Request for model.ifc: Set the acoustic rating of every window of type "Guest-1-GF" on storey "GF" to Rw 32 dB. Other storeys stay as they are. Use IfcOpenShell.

First a look at what the model holds.

```python
import ifcopenshell
import ifcopenshell.util.element

model = ifcopenshell.open("model.ifc")
print(model.schema)
storey = next(s for s in model.by_type("IfcBuildingStorey") if s.Name == "GF")
windows = [e for e in ifcopenshell.util.element.get_decomposition(storey) if e.is_a("IfcWindow")]
seen = {}
for e in windows:
    element_type = ifcopenshell.util.element.get_type(e)
    key = (element_type.Name if element_type != e and element_type else None, ifcopenshell.util.element.get_pset(e, "Pset_WindowCommon", "AcousticRating"))
    seen[key] = seen.get(key, 0) + 1
for (name, value), count in sorted(seen.items(), key=str):
    print(count, "x", name, "|", value)
```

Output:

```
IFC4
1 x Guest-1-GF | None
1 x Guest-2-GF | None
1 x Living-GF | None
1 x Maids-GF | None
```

```python
import ifcopenshell
import ifcopenshell.api.pset
import ifcopenshell.util.element

model = ifcopenshell.open("model.ifc")

storey = next(s for s in model.by_type("IfcBuildingStorey") if s.Name == "GF")
windows = [e for e in ifcopenshell.util.element.get_decomposition(storey) if e.is_a("IfcWindow")]

count = 0
for e in windows:
    element_type = ifcopenshell.util.element.get_type(e)
    if element_type in (None, e) or element_type.Name != "Guest-1-GF":
        continue
    # add_pset returns the element's existing set when there is one.
    pset = ifcopenshell.api.pset.add_pset(model, product=e, name="Pset_WindowCommon")
    ifcopenshell.api.pset.edit_pset(model, pset=pset, properties={"AcousticRating": "Rw 32 dB"})
    count += 1

print(count, "windows updated")

model.write("model_v2.ifc")
```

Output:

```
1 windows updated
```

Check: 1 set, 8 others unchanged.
